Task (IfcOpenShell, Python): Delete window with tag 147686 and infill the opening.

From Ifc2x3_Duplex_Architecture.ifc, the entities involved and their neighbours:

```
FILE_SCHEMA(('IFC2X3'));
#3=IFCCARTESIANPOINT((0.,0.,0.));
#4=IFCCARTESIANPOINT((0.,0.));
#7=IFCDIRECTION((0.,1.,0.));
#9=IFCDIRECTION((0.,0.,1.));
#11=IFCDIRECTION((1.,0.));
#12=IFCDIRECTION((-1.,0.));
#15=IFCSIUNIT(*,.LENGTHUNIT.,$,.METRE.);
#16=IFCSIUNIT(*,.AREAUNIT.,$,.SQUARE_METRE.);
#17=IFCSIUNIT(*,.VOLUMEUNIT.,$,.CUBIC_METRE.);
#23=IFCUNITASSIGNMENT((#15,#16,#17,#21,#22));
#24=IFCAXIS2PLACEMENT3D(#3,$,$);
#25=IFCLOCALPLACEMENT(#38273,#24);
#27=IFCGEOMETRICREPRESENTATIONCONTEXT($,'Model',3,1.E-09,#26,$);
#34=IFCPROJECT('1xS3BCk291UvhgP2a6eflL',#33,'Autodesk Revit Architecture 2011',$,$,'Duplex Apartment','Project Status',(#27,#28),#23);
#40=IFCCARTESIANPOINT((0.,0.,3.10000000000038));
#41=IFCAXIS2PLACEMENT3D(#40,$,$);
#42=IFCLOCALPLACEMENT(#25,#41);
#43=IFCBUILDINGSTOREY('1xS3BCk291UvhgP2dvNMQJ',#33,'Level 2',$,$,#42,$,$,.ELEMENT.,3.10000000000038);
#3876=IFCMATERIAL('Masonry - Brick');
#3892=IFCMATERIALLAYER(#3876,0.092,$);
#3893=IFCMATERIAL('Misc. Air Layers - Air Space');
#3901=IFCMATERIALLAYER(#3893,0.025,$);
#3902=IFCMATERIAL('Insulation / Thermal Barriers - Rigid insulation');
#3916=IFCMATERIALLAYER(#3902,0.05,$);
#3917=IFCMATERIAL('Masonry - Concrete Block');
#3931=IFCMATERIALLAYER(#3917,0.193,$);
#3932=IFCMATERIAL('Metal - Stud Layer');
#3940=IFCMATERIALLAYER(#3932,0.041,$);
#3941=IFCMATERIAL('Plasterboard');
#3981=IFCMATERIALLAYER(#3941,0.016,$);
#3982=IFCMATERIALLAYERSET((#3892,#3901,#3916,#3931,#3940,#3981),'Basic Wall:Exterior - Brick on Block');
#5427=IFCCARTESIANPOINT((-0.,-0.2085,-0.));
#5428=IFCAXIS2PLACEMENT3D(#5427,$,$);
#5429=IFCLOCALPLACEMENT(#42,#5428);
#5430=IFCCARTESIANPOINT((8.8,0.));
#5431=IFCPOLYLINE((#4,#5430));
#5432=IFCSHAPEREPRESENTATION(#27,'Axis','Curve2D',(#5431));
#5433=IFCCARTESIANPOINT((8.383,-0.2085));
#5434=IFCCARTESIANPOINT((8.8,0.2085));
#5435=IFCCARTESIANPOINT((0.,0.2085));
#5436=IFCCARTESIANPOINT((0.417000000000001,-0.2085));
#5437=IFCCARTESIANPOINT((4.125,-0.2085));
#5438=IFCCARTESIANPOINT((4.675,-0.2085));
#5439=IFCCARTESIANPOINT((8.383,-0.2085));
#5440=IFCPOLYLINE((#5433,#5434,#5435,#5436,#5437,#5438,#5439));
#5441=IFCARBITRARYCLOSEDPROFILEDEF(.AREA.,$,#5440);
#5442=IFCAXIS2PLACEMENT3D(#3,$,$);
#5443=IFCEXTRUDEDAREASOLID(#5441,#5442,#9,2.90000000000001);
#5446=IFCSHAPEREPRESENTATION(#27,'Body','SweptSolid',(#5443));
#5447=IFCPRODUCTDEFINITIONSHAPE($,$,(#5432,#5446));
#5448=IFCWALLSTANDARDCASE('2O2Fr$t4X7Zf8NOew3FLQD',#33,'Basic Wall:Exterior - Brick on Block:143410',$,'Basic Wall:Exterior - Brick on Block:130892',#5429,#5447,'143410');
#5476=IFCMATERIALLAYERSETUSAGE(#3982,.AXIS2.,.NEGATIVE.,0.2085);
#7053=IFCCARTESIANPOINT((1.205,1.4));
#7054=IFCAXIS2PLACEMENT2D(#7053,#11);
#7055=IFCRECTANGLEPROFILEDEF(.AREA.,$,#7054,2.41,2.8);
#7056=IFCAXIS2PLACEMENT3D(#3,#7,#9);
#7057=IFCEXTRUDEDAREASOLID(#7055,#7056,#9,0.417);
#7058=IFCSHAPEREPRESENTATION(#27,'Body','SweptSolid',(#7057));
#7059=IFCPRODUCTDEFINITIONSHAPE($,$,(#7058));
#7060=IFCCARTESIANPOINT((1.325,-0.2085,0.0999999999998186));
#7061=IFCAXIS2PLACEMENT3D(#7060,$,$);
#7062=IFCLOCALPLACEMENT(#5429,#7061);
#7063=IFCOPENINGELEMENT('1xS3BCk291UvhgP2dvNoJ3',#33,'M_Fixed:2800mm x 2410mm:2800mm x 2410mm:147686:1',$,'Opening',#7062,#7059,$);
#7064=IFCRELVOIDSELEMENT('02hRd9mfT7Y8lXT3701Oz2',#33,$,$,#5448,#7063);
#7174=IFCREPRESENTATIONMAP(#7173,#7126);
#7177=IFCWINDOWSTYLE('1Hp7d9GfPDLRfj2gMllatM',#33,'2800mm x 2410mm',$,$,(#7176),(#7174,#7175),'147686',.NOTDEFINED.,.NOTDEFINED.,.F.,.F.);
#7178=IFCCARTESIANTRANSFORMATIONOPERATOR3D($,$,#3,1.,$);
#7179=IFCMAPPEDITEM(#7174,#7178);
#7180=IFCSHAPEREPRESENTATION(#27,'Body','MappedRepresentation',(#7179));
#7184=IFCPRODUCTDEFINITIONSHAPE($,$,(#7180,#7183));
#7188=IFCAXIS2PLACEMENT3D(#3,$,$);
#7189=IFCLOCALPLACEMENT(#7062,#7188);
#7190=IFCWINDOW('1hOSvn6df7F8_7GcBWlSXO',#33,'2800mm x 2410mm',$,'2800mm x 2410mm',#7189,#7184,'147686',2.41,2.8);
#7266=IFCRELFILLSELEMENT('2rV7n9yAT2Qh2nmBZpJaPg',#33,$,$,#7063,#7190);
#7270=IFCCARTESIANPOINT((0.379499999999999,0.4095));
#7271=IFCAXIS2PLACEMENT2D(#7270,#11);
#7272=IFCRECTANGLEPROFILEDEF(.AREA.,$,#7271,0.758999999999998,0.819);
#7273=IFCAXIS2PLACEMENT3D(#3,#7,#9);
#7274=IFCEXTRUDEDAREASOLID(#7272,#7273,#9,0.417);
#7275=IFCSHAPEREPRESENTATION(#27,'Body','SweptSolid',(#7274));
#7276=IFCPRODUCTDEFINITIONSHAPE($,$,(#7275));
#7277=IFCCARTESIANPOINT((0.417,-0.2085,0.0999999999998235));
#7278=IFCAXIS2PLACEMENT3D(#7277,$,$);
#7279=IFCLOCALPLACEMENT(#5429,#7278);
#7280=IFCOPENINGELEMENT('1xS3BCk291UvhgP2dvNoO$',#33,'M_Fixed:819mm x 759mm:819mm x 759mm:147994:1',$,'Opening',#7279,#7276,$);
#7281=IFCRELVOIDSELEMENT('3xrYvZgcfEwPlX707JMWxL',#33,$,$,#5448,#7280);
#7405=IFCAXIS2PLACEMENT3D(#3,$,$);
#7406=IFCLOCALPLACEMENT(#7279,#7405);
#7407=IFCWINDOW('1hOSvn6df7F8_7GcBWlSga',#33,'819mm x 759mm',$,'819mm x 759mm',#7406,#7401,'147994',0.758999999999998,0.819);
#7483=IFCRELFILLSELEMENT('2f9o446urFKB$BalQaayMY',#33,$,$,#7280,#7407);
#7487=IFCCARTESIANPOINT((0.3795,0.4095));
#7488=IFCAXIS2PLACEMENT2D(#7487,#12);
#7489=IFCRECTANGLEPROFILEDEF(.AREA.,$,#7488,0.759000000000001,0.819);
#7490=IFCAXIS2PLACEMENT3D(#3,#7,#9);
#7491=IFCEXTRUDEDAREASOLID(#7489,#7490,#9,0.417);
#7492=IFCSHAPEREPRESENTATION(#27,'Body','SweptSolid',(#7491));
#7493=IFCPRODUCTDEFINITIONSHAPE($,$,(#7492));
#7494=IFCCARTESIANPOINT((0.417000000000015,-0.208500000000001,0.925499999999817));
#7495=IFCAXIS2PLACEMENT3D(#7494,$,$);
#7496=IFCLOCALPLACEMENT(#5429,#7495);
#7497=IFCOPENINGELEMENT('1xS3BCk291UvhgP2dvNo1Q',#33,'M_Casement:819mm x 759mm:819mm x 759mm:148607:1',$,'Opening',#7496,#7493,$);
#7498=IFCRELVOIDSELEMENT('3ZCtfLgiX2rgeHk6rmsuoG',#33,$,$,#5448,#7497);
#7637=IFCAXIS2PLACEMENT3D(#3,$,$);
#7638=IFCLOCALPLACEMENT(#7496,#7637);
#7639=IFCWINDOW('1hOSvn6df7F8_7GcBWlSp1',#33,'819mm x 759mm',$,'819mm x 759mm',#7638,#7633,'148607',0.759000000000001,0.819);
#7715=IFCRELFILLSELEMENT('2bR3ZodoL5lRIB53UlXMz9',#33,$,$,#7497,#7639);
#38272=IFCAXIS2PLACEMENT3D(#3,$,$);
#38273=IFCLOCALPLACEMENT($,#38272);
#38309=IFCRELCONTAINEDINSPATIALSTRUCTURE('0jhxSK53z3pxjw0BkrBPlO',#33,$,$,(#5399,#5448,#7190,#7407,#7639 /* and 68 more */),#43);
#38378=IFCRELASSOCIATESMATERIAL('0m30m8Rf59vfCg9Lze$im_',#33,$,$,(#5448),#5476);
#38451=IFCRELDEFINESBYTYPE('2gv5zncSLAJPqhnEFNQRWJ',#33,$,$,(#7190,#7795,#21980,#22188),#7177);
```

```python
import ifcopenshell
import ifcopenshell.api.feature
import ifcopenshell.api.root
import ifcopenshell.geom
import ifcopenshell.util.shape

model = ifcopenshell.open("Ifc2x3_Duplex_Architecture.ifc")
settings = ifcopenshell.geom.settings()


def volume(element):
    """Net volume in cubic metres, openings subtracted."""
    shape = ifcopenshell.geom.create_shape(settings, element)
    return ifcopenshell.util.shape.get_volume(shape.geometry)


window = model.by_guid("1hOSvn6df7F8_7GcBWlSXO")
opening = window.FillsVoids[0].RelatingOpeningElement
wall = opening.VoidsElements[0].RelatingBuildingElement
before = volume(wall)

ifcopenshell.api.root.remove_product(model, product=window)
ifcopenshell.api.feature.remove_feature(model, feature=opening)

after = volume(wall)

print(f"wall volume {before:.3f} -> {after:.3f} m3")

model.write("Ifc2x3_Duplex_Architecture_edited.ifc")
```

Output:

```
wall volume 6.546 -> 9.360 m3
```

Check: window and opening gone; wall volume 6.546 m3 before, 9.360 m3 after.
